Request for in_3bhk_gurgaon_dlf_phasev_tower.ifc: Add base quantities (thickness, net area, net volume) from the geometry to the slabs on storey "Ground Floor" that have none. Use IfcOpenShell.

First a look at what the model holds.

```python
import ifcopenshell
import ifcopenshell.util.element
import ifcopenshell.util.unit

model = ifcopenshell.open("in_3bhk_gurgaon_dlf_phasev_tower.ifc")
print(model.schema)
for unit_type in ("LENGTHUNIT", "AREAUNIT", "VOLUMEUNIT"):
    print(unit_type, ifcopenshell.util.unit.calculate_unit_scale(model, unit_type))
storey = next(s for s in model.by_type("IfcBuildingStorey") if s.Name == "Ground Floor")
slabs = [e for e in ifcopenshell.util.element.get_decomposition(storey) if e.is_a("IfcSlab")]
for e in sorted(slabs, key=lambda e: e.id()):
    print(e.id(), e.is_a(), e.Name, list(ifcopenshell.util.element.get_psets(e, qtos_only=True)), sep=" | ")
```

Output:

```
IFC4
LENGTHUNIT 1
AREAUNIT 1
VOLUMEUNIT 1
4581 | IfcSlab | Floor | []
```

```python
import ifcopenshell
import ifcopenshell.api.pset
import ifcopenshell.geom
import ifcopenshell.util.element
import ifcopenshell.util.shape
import ifcopenshell.util.unit

model = ifcopenshell.open("in_3bhk_gurgaon_dlf_phasev_tower.ifc")
unit_scale = ifcopenshell.util.unit.calculate_unit_scale(model)
area_scale = ifcopenshell.util.unit.calculate_unit_scale(model, "AREAUNIT")
volume_scale = ifcopenshell.util.unit.calculate_unit_scale(model, "VOLUMEUNIT")
settings = ifcopenshell.geom.settings()

storey = next(s for s in model.by_type("IfcBuildingStorey") if s.Name == "Ground Floor")
slabs = [e for e in ifcopenshell.util.element.get_decomposition(storey) if e.is_a("IfcSlab")]

for e in sorted(slabs, key=lambda e: e.id()):
    if ifcopenshell.util.element.get_psets(e, qtos_only=True, should_inherit=False):
        continue
    # Geometry comes back in metres, in the element's own axes.
    shape = ifcopenshell.geom.create_shape(settings, e)
    values = {
        "Width": ifcopenshell.util.shape.get_z(shape.geometry) / unit_scale,
        "NetArea": ifcopenshell.util.shape.get_footprint_area(shape.geometry) / area_scale,
        "NetVolume": ifcopenshell.util.shape.get_volume(shape.geometry) / volume_scale,
    }
    qto = ifcopenshell.api.pset.add_qto(model, product=e, name="Qto_SlabBaseQuantities")
    ifcopenshell.api.pset.edit_qto(model, qto=qto, properties=values)
    print(e.id(), {k: round(v, 3) for k, v in values.items()})

model.write("in_3bhk_gurgaon_dlf_phasev_tower_rev.ifc")
```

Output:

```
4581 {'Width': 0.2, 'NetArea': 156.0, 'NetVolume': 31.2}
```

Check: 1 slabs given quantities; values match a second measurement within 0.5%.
